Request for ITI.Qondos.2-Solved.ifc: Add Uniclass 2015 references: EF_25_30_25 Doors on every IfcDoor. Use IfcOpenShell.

First a look at what the model holds.

```python
import ifcopenshell

model = ifcopenshell.open("ITI.Qondos.2-Solved.ifc")
print(model.schema)
print("classifications:", [c.Name for c in model.by_type("IfcClassification")])
for ifc_class in ("IfcDoor", "IfcRoof", "IfcStair", "IfcWall", "IfcWindow"):
    print(ifc_class, len(model.by_type(ifc_class)))
```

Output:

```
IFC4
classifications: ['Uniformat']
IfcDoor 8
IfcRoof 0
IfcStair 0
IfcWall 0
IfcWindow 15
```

```python
import ifcopenshell
import ifcopenshell.api.classification

model = ifcopenshell.open("ITI.Qondos.2-Solved.ifc")

system = ifcopenshell.api.classification.add_classification(model, classification="Uniclass 2015")

codes = {
    "IfcDoor": ("EF_25_30_25", "Doors"),
}
for ifc_class, (code, name) in codes.items():
    products = model.by_type(ifc_class)
    ifcopenshell.api.classification.add_reference(
        model, products=products, classification=system, identification=code, name=name
    )
    print(code, len(products))

model.write("ITI.Qondos.2-Solved_rev.ifc")
```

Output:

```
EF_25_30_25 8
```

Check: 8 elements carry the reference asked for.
